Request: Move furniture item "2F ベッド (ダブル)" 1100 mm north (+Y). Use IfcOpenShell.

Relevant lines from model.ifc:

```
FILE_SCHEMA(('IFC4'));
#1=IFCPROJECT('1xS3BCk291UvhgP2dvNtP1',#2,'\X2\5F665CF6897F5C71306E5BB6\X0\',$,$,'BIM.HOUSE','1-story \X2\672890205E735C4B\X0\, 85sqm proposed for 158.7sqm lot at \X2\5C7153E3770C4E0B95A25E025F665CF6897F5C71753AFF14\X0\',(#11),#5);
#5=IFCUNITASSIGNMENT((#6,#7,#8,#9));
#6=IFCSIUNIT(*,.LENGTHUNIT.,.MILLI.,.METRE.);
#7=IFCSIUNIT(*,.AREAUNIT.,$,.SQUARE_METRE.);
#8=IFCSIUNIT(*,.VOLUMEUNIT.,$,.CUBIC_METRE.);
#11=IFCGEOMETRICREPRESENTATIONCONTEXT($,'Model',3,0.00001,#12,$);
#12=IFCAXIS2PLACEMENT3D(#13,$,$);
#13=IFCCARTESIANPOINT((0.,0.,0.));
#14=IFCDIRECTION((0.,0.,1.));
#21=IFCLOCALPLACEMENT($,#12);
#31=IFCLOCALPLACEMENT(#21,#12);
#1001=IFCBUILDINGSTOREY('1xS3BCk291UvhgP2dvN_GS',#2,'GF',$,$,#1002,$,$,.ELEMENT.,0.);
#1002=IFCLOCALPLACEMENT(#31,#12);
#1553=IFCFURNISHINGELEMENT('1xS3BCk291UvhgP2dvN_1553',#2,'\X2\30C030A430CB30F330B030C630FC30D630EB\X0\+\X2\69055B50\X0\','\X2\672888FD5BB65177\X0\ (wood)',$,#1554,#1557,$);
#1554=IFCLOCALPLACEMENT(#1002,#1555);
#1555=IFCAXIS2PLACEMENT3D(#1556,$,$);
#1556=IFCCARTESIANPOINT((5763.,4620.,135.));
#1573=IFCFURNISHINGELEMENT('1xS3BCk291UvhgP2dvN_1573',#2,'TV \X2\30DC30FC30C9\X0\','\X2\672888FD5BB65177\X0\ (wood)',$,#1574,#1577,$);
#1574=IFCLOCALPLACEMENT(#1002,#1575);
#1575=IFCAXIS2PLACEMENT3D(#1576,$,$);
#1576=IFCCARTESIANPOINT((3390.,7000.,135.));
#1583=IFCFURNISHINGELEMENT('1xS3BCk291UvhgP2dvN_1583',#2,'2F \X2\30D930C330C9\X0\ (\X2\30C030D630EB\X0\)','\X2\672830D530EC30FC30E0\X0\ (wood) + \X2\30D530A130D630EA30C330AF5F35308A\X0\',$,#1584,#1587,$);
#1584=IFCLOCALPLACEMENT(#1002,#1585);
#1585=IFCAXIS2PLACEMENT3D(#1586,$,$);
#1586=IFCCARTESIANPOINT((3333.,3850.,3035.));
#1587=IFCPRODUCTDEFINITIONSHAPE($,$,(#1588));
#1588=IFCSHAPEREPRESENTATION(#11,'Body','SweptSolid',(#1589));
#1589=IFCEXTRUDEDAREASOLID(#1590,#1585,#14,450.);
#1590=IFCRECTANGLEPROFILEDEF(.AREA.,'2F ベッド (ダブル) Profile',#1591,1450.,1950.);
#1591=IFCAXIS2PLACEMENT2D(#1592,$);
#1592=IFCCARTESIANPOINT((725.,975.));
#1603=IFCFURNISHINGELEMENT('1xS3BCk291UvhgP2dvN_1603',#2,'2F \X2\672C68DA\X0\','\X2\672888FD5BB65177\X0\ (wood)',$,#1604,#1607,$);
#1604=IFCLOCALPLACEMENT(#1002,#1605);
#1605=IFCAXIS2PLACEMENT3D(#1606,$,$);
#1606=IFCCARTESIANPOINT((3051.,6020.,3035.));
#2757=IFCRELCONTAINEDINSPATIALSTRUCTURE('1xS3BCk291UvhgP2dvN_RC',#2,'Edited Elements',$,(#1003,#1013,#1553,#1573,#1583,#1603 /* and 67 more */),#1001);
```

```python
import ifcopenshell
import ifcopenshell.api.geometry
import ifcopenshell.util.placement

model = ifcopenshell.open("model.ifc")

item = model.by_guid("1xS3BCk291UvhgP2dvN_1583")
matrix = ifcopenshell.util.placement.get_local_placement(item.ObjectPlacement)
matrix[1, 3] += 1100.0
ifcopenshell.api.geometry.edit_object_placement(model, product=item, matrix=matrix, is_si=False)

print(ifcopenshell.util.placement.get_local_placement(item.ObjectPlacement).round(3) + 0.0)

model.write("model_v2.ifc")
```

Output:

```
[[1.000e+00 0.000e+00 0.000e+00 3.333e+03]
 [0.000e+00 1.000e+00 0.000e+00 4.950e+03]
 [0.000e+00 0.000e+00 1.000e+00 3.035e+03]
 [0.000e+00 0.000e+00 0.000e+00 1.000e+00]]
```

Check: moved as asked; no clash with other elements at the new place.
